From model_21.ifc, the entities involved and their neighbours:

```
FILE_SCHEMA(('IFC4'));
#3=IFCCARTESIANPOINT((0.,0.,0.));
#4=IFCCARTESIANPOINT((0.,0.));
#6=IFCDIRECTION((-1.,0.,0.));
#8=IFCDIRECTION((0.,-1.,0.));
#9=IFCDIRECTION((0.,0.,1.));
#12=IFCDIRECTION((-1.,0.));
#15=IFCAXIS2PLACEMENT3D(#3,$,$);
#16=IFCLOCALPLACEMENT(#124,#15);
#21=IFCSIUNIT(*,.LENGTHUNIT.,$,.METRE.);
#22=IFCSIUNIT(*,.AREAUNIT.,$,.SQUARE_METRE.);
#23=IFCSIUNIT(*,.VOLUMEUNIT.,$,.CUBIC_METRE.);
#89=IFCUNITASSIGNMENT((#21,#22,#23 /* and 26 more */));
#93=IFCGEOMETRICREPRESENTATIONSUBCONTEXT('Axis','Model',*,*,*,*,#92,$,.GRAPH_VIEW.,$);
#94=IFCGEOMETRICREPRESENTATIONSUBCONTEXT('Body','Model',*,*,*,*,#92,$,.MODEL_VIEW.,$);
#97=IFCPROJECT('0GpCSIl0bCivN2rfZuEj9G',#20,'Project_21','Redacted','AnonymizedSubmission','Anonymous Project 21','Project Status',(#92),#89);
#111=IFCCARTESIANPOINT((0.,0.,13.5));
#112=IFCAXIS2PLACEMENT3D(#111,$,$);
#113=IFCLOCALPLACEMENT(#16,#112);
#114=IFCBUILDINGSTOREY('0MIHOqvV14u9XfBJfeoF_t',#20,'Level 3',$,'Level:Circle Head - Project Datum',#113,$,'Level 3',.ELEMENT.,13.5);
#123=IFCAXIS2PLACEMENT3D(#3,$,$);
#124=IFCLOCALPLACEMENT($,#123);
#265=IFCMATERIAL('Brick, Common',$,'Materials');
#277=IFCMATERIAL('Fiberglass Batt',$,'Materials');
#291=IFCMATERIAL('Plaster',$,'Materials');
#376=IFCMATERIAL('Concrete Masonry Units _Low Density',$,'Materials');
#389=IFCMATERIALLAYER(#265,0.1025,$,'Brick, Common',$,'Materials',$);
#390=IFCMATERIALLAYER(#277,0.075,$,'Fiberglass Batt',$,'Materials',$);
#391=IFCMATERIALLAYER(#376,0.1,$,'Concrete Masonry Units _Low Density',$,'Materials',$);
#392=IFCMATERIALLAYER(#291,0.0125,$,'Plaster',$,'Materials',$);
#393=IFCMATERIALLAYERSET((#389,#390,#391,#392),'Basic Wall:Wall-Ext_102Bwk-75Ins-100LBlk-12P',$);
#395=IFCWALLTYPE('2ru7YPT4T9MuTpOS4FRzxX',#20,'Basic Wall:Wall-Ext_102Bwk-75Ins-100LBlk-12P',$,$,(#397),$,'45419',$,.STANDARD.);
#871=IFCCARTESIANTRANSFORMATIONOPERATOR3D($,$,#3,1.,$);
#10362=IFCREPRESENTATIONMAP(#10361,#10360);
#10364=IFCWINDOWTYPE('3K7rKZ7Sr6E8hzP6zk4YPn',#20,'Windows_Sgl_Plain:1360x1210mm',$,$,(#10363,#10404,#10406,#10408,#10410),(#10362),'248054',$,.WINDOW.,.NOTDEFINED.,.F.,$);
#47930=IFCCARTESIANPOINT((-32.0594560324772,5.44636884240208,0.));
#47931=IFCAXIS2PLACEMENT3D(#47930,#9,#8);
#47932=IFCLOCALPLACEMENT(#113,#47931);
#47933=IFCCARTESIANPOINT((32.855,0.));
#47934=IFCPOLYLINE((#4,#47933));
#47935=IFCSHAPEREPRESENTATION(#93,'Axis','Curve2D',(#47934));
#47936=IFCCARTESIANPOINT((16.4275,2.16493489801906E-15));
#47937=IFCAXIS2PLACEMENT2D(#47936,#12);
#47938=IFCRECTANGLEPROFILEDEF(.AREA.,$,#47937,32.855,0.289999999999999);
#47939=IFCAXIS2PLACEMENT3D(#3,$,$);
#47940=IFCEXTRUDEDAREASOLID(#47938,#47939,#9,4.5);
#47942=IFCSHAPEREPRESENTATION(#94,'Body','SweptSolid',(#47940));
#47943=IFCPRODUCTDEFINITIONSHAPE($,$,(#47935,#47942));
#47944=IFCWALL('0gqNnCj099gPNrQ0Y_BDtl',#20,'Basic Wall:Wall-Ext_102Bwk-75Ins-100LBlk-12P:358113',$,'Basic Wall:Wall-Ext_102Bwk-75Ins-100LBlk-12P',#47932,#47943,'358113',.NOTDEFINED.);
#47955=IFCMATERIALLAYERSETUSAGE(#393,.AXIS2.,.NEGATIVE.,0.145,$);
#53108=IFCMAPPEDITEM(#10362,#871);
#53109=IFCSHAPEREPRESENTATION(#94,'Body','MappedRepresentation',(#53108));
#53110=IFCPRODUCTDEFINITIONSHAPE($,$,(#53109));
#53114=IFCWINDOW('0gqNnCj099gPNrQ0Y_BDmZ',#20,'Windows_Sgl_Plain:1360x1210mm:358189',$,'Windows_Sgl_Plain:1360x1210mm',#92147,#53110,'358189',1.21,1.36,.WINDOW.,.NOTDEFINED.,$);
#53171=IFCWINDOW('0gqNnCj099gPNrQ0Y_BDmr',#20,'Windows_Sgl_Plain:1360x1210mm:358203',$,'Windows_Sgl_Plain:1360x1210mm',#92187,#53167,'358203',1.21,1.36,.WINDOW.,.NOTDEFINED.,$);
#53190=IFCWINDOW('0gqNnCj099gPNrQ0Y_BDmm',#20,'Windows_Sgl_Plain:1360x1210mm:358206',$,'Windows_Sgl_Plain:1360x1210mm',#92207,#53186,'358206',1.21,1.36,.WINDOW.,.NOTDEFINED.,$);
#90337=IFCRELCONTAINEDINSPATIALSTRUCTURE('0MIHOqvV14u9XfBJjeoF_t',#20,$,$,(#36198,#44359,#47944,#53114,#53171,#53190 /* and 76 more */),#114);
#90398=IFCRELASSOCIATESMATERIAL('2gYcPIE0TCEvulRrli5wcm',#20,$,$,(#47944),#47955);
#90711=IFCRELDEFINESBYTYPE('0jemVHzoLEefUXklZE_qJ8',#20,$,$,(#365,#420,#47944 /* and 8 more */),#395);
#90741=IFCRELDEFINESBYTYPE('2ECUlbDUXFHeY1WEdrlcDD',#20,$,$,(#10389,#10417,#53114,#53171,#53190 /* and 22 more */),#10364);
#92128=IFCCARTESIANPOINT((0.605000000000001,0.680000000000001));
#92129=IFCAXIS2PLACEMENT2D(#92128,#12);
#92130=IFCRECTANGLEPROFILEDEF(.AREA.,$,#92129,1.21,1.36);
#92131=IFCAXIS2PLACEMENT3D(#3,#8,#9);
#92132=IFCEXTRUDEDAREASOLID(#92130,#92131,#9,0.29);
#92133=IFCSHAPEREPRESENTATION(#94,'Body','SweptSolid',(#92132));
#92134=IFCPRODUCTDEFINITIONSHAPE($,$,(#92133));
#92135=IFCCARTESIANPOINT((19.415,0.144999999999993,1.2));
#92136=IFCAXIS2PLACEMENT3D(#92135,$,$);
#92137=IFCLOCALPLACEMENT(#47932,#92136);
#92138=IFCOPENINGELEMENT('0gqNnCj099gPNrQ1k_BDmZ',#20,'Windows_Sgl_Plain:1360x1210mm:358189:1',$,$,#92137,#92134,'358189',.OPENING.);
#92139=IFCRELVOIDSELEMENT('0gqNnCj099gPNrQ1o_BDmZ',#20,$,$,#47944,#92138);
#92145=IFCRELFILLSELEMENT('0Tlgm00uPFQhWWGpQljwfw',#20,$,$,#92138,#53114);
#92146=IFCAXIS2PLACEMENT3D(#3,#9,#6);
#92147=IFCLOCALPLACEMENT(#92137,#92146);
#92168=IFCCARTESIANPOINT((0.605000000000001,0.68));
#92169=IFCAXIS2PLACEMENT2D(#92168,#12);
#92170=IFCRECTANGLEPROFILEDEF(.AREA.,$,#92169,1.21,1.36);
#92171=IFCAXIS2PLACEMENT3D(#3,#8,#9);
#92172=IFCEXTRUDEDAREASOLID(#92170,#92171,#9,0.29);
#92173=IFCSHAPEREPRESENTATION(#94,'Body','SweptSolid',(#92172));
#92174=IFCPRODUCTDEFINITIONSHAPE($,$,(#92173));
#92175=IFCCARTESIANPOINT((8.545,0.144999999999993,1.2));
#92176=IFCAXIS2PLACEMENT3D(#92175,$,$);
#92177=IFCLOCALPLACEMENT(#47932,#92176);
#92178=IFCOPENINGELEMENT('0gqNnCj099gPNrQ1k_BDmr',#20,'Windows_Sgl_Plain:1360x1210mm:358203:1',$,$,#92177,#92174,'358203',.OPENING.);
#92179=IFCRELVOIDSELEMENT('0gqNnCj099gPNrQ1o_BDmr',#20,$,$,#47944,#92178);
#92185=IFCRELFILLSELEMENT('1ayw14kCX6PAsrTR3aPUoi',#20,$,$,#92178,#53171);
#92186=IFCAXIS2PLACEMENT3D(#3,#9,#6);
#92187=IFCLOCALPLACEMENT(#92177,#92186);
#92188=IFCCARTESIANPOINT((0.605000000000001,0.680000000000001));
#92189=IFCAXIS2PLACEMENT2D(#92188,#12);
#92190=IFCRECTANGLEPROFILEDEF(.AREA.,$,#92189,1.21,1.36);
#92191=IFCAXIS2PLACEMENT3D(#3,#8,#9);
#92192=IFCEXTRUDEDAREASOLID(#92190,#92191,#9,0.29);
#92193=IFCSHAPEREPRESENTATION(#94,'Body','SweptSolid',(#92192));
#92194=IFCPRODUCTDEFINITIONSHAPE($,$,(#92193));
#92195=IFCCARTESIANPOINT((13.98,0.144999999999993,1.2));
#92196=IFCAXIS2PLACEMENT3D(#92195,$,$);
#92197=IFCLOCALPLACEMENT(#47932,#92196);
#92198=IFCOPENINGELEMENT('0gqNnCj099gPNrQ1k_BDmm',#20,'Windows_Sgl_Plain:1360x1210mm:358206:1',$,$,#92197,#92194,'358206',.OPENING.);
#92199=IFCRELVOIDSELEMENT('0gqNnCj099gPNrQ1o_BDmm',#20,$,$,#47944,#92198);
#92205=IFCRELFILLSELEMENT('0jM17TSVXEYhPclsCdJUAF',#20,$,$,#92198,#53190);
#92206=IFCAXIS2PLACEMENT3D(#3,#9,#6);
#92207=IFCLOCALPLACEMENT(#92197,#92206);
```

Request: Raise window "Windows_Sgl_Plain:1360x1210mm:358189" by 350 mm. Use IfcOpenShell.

```python
import numpy as np
import ifcopenshell
import ifcopenshell.api.geometry
import ifcopenshell.util.placement
import ifcopenshell.util.unit

model = ifcopenshell.open("model_21.ifc")
unit_scale = ifcopenshell.util.unit.calculate_unit_scale(model)

window = model.by_id(53114)
opening = window.FillsVoids[0].RelatingOpeningElement
dz = 0.35 / unit_scale

shift = np.array([0.0, 0.0, dz])
# The window is placed relative to its opening, so it follows when the opening moves.
matrix = ifcopenshell.util.placement.get_local_placement(opening.ObjectPlacement)
matrix[:3, 3] += shift
ifcopenshell.api.geometry.edit_object_placement(
    model, product=opening, matrix=matrix, is_si=False, should_transform_children=True
)

print(f"moved by {dz * unit_scale:+.3f} m")

model.write("model_21_edited.ifc")
```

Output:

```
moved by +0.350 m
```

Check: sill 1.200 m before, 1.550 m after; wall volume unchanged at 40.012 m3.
